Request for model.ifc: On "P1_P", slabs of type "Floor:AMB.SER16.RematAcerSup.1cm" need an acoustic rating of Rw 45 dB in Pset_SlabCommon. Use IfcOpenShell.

First a look at what the model holds.

```python
import ifcopenshell
import ifcopenshell.util.element

model = ifcopenshell.open("model.ifc")
print(model.schema)
storey = next(s for s in model.by_type("IfcBuildingStorey") if s.Name == "P1_P")
slabs = [e for e in ifcopenshell.util.element.get_decomposition(storey) if e.is_a("IfcSlab")]
seen = {}
for e in slabs:
    element_type = ifcopenshell.util.element.get_type(e)
    key = (element_type.Name if element_type != e and element_type else None, ifcopenshell.util.element.get_pset(e, "Pset_SlabCommon", "AcousticRating"))
    seen[key] = seen.get(key, 0) + 1
for (name, value), count in sorted(seen.items(), key=str):
    print(count, "x", name, "|", value)
```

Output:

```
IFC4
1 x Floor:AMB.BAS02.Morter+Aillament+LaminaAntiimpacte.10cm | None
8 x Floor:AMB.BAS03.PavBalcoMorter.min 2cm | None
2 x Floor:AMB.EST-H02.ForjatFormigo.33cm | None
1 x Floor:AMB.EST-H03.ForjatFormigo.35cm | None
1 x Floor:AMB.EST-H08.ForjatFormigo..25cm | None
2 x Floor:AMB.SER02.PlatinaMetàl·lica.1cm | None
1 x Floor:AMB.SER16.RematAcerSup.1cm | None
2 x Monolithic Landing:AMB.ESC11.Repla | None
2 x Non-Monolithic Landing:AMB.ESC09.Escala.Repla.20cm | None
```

```python
import ifcopenshell
import ifcopenshell.api.pset
import ifcopenshell.util.element

model = ifcopenshell.open("model.ifc")

storey = next(s for s in model.by_type("IfcBuildingStorey") if s.Name == "P1_P")
slabs = [e for e in ifcopenshell.util.element.get_decomposition(storey) if e.is_a("IfcSlab")]

count = 0
for e in slabs:
    element_type = ifcopenshell.util.element.get_type(e)
    if element_type in (None, e) or element_type.Name != "Floor:AMB.SER16.RematAcerSup.1cm":
        continue
    # add_pset returns the element's existing set when there is one.
    pset = ifcopenshell.api.pset.add_pset(model, product=e, name="Pset_SlabCommon")
    ifcopenshell.api.pset.edit_pset(model, pset=pset, properties={"AcousticRating": "Rw 45 dB"})
    count += 1

print(count, "slabs updated")

model.write("model_v2.ifc")
```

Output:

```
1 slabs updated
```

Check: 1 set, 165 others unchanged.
